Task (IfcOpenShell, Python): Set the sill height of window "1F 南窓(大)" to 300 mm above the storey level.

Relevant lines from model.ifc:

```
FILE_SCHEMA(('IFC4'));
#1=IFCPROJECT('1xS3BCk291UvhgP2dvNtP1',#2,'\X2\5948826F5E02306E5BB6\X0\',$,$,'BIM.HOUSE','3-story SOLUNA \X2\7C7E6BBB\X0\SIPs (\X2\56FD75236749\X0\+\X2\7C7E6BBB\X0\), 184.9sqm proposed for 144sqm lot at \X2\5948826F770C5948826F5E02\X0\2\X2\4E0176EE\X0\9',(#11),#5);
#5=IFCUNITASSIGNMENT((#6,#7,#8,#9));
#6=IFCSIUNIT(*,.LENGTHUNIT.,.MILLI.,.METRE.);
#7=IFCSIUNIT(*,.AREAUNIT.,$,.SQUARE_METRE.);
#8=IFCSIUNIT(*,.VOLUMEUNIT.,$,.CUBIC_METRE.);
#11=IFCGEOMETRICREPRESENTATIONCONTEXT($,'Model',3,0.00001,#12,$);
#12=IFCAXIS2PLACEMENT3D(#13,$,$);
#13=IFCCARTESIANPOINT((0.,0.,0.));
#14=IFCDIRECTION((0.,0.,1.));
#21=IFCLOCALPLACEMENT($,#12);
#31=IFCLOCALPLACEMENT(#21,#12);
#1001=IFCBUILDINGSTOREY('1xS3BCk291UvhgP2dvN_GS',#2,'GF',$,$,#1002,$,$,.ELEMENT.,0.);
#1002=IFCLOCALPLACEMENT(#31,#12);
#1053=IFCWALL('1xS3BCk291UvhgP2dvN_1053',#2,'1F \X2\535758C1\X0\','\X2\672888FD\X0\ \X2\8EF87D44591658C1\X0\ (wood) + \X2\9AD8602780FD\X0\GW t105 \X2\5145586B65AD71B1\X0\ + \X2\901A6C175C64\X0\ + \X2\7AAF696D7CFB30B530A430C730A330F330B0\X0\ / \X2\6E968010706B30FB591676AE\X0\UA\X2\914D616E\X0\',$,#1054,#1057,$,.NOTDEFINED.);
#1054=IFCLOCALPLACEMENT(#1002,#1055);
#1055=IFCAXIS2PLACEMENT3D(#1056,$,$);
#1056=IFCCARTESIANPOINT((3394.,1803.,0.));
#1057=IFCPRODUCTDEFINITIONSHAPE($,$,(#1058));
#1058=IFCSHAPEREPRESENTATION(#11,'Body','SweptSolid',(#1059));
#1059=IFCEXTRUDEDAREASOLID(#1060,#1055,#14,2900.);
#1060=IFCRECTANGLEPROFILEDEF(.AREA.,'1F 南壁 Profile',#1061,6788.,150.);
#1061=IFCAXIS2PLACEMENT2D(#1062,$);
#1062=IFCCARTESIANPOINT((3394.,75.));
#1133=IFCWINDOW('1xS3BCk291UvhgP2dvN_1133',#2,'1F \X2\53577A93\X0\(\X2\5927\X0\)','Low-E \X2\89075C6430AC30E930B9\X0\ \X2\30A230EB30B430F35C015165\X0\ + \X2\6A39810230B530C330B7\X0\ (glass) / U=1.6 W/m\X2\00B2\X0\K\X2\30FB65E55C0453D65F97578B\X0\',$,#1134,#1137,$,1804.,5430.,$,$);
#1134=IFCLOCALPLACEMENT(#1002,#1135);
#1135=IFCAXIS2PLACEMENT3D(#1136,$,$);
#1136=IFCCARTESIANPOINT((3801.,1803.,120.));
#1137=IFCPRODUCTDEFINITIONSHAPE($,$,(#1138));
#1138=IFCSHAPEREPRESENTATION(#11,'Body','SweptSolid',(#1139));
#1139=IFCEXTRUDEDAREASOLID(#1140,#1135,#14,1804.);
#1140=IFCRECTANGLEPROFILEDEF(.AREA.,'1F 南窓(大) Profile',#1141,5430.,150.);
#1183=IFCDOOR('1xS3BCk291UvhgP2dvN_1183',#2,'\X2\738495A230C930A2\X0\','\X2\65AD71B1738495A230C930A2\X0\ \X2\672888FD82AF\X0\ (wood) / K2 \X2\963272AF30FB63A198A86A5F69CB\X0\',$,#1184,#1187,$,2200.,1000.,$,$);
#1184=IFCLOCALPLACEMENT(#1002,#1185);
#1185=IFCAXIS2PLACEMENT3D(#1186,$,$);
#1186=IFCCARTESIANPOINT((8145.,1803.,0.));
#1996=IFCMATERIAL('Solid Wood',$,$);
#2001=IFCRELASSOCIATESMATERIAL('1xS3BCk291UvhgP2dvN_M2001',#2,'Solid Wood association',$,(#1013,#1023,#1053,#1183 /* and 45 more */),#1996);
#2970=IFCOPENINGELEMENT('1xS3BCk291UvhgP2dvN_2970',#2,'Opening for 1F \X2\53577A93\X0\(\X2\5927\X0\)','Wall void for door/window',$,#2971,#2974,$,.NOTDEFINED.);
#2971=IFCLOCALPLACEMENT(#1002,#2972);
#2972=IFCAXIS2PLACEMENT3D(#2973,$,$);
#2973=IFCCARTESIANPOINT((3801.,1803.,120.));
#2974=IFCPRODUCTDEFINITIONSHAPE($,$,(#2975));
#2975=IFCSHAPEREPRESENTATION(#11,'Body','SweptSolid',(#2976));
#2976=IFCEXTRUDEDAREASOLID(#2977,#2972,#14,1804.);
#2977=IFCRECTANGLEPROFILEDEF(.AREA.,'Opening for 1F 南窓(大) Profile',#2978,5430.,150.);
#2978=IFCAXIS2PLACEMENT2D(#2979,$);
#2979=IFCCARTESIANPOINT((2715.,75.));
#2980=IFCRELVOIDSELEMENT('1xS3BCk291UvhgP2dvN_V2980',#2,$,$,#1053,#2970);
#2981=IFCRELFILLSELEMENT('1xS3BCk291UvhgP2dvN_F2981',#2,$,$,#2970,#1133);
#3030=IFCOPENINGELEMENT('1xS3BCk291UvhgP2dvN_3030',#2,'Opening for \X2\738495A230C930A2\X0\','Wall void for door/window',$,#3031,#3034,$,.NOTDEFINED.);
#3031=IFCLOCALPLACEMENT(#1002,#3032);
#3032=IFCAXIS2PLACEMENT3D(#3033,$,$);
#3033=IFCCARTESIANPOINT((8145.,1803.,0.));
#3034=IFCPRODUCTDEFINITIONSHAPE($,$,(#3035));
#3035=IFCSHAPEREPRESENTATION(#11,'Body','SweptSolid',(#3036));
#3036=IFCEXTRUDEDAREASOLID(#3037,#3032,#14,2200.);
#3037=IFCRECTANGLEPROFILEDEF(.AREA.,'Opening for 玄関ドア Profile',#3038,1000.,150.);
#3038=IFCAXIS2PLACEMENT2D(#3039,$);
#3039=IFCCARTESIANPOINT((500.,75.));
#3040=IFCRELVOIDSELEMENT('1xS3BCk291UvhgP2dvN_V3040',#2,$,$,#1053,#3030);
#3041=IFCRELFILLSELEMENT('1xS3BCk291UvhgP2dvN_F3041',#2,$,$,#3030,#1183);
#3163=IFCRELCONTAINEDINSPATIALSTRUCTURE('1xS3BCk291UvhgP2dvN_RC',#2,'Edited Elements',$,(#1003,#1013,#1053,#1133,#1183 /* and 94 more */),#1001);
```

```python
import numpy as np
import ifcopenshell
import ifcopenshell.api.geometry
import ifcopenshell.geom
import ifcopenshell.util.element
import ifcopenshell.util.placement
import ifcopenshell.util.shape
import ifcopenshell.util.unit

model = ifcopenshell.open("model.ifc")
unit_scale = ifcopenshell.util.unit.calculate_unit_scale(model)

window = model.by_guid("1xS3BCk291UvhgP2dvN_1133")
opening = window.FillsVoids[0].RelatingOpeningElement
storey = ifcopenshell.util.element.get_container(window, ifc_class="IfcBuildingStorey")
level = ifcopenshell.util.placement.get_local_placement(storey.ObjectPlacement)[2, 3]

# The opening's origin need not be at the sill, so measure its lowest point.
shape = ifcopenshell.geom.create_shape(ifcopenshell.geom.settings(), opening)
bottom = ifcopenshell.util.shape.get_shape_bottom_elevation(shape, shape.geometry) / unit_scale
dz = level + 0.3 / unit_scale - bottom

shift = np.array([0.0, 0.0, dz])
# The window is not placed relative to its opening, so move both.
for product in (opening, window):
    matrix = ifcopenshell.util.placement.get_local_placement(product.ObjectPlacement)
    matrix[:3, 3] += shift
    ifcopenshell.api.geometry.edit_object_placement(model, product=product, matrix=matrix, is_si=False)

print(f"moved by {dz * unit_scale:+.3f} m")

model.write("model_v2.ifc")
```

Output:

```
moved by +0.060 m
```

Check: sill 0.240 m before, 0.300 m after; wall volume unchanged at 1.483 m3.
